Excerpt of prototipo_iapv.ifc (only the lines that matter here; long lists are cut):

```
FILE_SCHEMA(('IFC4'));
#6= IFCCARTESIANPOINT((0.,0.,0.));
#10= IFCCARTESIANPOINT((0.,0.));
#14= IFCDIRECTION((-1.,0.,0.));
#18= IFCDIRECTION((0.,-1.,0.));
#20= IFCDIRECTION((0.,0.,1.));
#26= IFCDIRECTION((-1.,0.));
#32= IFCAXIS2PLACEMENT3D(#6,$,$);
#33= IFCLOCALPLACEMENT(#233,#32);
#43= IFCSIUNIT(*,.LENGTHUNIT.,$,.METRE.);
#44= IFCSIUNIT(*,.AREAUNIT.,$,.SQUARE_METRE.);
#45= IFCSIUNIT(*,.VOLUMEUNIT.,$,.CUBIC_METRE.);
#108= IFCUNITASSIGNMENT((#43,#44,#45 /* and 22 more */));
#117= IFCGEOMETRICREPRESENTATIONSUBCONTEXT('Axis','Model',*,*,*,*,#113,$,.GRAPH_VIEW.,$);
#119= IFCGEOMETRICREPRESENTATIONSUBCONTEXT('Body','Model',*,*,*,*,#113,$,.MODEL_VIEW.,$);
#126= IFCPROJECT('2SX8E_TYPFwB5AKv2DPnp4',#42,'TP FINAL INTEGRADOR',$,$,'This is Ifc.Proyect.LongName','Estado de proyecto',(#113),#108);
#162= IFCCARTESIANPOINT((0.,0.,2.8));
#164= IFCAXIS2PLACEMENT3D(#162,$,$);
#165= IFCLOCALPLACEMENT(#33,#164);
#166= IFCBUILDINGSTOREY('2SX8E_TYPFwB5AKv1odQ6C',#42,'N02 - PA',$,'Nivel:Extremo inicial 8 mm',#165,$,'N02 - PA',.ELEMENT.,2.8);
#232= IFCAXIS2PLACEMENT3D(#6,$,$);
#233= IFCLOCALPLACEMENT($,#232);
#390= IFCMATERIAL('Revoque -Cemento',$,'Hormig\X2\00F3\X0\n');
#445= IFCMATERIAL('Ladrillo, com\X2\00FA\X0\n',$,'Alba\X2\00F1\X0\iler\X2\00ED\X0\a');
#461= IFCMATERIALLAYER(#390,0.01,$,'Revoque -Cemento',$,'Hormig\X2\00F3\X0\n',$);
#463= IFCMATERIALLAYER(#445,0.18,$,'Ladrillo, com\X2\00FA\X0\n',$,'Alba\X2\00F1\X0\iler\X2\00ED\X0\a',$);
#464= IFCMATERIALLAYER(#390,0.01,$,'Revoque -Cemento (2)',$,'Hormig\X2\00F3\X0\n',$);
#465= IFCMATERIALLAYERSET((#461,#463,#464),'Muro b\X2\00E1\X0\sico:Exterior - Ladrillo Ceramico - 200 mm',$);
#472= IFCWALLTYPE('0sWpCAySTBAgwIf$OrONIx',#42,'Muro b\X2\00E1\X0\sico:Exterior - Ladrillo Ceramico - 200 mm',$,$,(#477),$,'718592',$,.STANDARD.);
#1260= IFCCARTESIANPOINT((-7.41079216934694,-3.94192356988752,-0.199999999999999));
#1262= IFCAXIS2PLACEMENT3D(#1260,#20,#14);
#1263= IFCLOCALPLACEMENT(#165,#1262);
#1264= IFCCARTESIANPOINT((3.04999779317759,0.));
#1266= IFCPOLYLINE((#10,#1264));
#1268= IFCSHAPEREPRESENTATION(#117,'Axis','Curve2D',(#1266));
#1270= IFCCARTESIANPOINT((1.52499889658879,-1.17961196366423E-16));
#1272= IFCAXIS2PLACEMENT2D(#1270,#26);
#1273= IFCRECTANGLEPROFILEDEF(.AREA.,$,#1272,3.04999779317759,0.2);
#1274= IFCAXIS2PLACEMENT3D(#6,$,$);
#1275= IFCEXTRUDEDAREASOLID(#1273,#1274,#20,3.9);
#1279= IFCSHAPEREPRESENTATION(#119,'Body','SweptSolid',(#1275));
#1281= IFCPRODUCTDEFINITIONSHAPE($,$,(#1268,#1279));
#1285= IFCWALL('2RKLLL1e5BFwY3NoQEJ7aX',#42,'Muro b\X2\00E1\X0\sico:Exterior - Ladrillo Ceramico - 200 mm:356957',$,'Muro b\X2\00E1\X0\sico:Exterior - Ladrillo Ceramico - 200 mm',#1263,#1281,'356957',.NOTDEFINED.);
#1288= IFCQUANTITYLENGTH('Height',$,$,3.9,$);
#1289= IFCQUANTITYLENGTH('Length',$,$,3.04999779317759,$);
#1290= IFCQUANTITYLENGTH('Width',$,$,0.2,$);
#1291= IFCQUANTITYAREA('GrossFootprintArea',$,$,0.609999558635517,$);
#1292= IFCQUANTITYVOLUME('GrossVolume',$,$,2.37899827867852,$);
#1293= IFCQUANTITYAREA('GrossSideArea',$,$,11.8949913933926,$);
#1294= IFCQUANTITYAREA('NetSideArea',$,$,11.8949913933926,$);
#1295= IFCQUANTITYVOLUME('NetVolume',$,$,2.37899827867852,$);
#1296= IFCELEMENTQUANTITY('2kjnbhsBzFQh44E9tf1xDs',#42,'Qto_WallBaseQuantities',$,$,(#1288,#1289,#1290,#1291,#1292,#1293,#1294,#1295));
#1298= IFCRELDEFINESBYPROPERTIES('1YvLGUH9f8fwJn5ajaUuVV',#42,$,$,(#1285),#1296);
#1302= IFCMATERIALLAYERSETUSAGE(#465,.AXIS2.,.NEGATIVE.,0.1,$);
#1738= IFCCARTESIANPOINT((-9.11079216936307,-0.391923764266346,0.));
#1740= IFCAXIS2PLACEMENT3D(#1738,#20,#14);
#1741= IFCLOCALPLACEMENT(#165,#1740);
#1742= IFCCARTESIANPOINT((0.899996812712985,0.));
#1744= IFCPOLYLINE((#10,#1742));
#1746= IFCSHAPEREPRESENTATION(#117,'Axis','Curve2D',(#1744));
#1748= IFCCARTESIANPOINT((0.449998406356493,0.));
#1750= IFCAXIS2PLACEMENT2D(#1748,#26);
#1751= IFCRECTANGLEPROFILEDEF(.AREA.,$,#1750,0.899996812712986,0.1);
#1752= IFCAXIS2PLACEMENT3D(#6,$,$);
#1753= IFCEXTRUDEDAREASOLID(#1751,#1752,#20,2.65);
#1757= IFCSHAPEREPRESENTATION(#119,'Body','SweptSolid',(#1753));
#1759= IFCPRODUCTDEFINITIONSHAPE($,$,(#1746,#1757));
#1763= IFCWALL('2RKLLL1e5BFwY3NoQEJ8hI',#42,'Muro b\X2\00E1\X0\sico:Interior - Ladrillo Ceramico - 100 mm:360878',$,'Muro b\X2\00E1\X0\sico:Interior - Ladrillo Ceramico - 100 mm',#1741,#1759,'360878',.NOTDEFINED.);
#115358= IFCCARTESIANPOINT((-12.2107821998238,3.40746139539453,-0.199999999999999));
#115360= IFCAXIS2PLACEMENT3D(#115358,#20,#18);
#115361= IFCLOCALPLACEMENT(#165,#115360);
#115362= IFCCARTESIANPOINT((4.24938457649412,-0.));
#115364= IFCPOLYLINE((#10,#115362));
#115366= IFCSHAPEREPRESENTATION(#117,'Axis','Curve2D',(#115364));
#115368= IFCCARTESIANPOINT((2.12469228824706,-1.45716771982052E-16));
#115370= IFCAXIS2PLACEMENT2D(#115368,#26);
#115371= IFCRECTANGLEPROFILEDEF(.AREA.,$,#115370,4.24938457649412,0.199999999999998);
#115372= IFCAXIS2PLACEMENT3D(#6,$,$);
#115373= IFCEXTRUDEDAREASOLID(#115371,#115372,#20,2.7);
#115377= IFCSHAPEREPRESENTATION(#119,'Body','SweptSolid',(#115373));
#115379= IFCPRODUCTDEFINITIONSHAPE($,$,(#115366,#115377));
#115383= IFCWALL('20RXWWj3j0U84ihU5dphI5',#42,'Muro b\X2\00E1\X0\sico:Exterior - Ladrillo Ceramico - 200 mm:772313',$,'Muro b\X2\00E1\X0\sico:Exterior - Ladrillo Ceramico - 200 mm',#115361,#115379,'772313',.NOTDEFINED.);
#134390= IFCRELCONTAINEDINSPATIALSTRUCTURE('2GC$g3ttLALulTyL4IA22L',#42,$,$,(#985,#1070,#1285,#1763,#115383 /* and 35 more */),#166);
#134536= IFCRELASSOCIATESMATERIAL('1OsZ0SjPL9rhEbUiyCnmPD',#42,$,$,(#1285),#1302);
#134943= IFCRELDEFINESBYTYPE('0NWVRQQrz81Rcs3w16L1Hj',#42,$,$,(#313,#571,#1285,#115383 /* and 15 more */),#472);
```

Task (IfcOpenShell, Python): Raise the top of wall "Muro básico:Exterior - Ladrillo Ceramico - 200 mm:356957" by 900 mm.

```python
import ifcopenshell
import ifcopenshell.api.pset
import ifcopenshell.geom
import ifcopenshell.util.element
import ifcopenshell.util.representation
import ifcopenshell.util.shape
import ifcopenshell.util.unit

model = ifcopenshell.open("prototipo_iapv.ifc")
unit_scale = ifcopenshell.util.unit.calculate_unit_scale(model)
area_scale = ifcopenshell.util.unit.calculate_unit_scale(model, "AREAUNIT")
volume_scale = ifcopenshell.util.unit.calculate_unit_scale(model, "VOLUMEUNIT")
settings = ifcopenshell.geom.settings()


def volume(element):
    """Net volume in cubic metres, openings subtracted."""
    shape = ifcopenshell.geom.create_shape(settings, element)
    return ifcopenshell.util.shape.get_volume(shape.geometry)


wall = model.by_guid("2RKLLL1e5BFwY3NoQEJ7aX")
before = volume(wall)

body = ifcopenshell.util.representation.get_representation(wall, "Model", "Body")
solid = body.Items[0]
old_height = solid.Depth
solid.Depth += 0.9 / unit_scale
after = volume(wall)
thickness = 0.2  # wall thickness in metres

# Update the stored height, areas and volumes.
qto = model.by_id(ifcopenshell.util.element.get_pset(wall, "Qto_WallBaseQuantities", should_inherit=False)["id"])
ifcopenshell.api.pset.edit_qto(model, qto=qto, properties={
    "Height": solid.Depth,
    "GrossVolume": ifcopenshell.util.element.get_pset(wall, "Qto_WallBaseQuantities", "GrossVolume") * solid.Depth / old_height,
    "GrossSideArea": ifcopenshell.util.element.get_pset(wall, "Qto_WallBaseQuantities", "GrossSideArea") * solid.Depth / old_height,
    "NetSideArea": after / thickness / area_scale,
    "NetVolume": after / volume_scale,
})

print(f"height {old_height:g} -> {solid.Depth:g}, volume {before:.3f} -> {after:.3f} m3")

model.write("prototipo_iapv_updated.ifc")
```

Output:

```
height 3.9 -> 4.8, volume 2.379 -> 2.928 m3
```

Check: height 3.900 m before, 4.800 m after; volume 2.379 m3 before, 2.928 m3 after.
